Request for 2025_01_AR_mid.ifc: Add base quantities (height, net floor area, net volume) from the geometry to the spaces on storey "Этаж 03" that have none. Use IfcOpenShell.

First a look at what the model holds.

```python
import ifcopenshell
import ifcopenshell.util.element
import ifcopenshell.util.unit

model = ifcopenshell.open("2025_01_AR_mid.ifc")
print(model.schema)
for unit_type in ("LENGTHUNIT", "AREAUNIT", "VOLUMEUNIT"):
    print(unit_type, ifcopenshell.util.unit.calculate_unit_scale(model, unit_type))
storey = next(s for s in model.by_type("IfcBuildingStorey") if s.Name == "Этаж 03")
spaces = [e for e in ifcopenshell.util.element.get_decomposition(storey) if e.is_a("IfcSpace")]
for e in sorted(spaces, key=lambda e: e.id()):
    print(e.id(), e.is_a(), e.Name, list(ifcopenshell.util.element.get_psets(e, qtos_only=True)), sep=" | ")
```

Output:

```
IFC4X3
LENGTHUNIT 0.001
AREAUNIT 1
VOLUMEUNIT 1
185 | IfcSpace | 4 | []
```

```python
import ifcopenshell
import ifcopenshell.api.pset
import ifcopenshell.geom
import ifcopenshell.util.element
import ifcopenshell.util.shape
import ifcopenshell.util.unit

model = ifcopenshell.open("2025_01_AR_mid.ifc")
unit_scale = ifcopenshell.util.unit.calculate_unit_scale(model)
area_scale = ifcopenshell.util.unit.calculate_unit_scale(model, "AREAUNIT")
volume_scale = ifcopenshell.util.unit.calculate_unit_scale(model, "VOLUMEUNIT")
settings = ifcopenshell.geom.settings()

storey = next(s for s in model.by_type("IfcBuildingStorey") if s.Name == "Этаж 03")
spaces = [e for e in ifcopenshell.util.element.get_decomposition(storey) if e.is_a("IfcSpace")]

for e in sorted(spaces, key=lambda e: e.id()):
    if ifcopenshell.util.element.get_psets(e, qtos_only=True, should_inherit=False):
        continue
    # Geometry comes back in metres, in the element's own axes.
    shape = ifcopenshell.geom.create_shape(settings, e)
    values = {
        "Height": ifcopenshell.util.shape.get_z(shape.geometry) / unit_scale,
        "NetFloorArea": ifcopenshell.util.shape.get_footprint_area(shape.geometry) / area_scale,
        "NetVolume": ifcopenshell.util.shape.get_volume(shape.geometry) / volume_scale,
    }
    qto = ifcopenshell.api.pset.add_qto(model, product=e, name="Qto_SpaceBaseQuantities")
    ifcopenshell.api.pset.edit_qto(model, qto=qto, properties=values)
    print(e.id(), {k: round(v, 3) for k, v in values.items()})

model.write("2025_01_AR_mid-out.ifc")
```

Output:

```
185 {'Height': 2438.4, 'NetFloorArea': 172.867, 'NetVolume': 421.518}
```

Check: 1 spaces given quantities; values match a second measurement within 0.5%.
